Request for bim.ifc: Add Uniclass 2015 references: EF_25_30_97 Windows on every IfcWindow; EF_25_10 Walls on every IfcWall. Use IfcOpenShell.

First a look at what the model holds.

```python
import ifcopenshell

model = ifcopenshell.open("bim.ifc")
print(model.schema)
print("classifications:", [c.Name for c in model.by_type("IfcClassification")])
for ifc_class in ("IfcDoor", "IfcRoof", "IfcStair", "IfcWall", "IfcWindow"):
    print(ifc_class, len(model.by_type(ifc_class)))
```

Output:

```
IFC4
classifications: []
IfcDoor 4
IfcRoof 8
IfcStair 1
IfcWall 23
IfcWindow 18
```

```python
import ifcopenshell
import ifcopenshell.api.classification

model = ifcopenshell.open("bim.ifc")

system = ifcopenshell.api.classification.add_classification(model, classification="Uniclass 2015")

codes = {
    "IfcWindow": ("EF_25_30_97", "Windows"),
    "IfcWall": ("EF_25_10", "Walls"),
}
for ifc_class, (code, name) in codes.items():
    products = model.by_type(ifc_class)
    ifcopenshell.api.classification.add_reference(
        model, products=products, classification=system, identification=code, name=name
    )
    print(code, len(products))

model.write("bim_v2.ifc")
```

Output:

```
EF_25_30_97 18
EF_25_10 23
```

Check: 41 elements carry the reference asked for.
